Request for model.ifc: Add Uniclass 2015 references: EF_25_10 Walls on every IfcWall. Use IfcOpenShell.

First a look at what the model holds.

```python
import ifcopenshell

model = ifcopenshell.open("model.ifc")
print(model.schema)
print("classifications:", [c.Name for c in model.by_type("IfcClassification")])
for ifc_class in ("IfcDoor", "IfcRoof", "IfcStair", "IfcWall", "IfcWindow"):
    print(ifc_class, len(model.by_type(ifc_class)))
```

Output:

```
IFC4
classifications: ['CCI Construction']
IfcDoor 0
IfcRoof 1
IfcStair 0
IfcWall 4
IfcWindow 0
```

```python
import ifcopenshell
import ifcopenshell.api.classification

model = ifcopenshell.open("model.ifc")

system = ifcopenshell.api.classification.add_classification(model, classification="Uniclass 2015")

codes = {
    "IfcWall": ("EF_25_10", "Walls"),
}
for ifc_class, (code, name) in codes.items():
    products = model.by_type(ifc_class)
    ifcopenshell.api.classification.add_reference(
        model, products=products, classification=system, identification=code, name=name
    )
    print(code, len(products))

model.write("model_rev.ifc")
```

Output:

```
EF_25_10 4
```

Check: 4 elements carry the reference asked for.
